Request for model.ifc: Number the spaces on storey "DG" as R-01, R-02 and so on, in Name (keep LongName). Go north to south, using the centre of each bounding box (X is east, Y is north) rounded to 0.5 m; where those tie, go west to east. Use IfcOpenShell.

First a look at what the model holds.

```python
import ifcopenshell
import ifcopenshell.util.element
import ifcopenshell.util.placement

model = ifcopenshell.open("model.ifc")
print(model.schema)
storey = next(s for s in model.by_type("IfcBuildingStorey") if s.Name == "DG")
spaces = [e for e in ifcopenshell.util.element.get_decomposition(storey) if e.is_a("IfcSpace")]
for e in sorted(spaces, key=lambda e: e.id()):
    origin = ifcopenshell.util.placement.get_local_placement(e.ObjectPlacement)[:3, 3]
    print(e.id(), e.Name, e.LongName, origin.round(2) + 0.0, sep=" | ")
```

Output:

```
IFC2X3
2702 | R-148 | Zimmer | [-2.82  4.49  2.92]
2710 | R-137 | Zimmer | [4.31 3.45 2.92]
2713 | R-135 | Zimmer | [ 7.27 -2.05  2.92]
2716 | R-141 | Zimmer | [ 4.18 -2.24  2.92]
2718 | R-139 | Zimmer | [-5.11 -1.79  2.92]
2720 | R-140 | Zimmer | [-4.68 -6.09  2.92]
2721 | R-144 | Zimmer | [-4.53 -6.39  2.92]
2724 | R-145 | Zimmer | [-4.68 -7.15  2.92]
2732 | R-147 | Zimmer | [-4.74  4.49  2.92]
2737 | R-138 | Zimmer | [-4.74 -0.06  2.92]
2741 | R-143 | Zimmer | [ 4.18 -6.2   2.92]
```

```python
import ifcopenshell
import ifcopenshell.geom
import ifcopenshell.util.element
import ifcopenshell.util.shape

model = ifcopenshell.open("model.ifc")
settings = ifcopenshell.geom.settings()
settings.set("use-world-coords", True)


def centre(element):
    shape = ifcopenshell.geom.create_shape(settings, element)
    return ifcopenshell.util.shape.get_bbox_centroid(shape.geometry)


storey = next(s for s in model.by_type("IfcBuildingStorey") if s.Name == "DG")
spaces = [e for e in ifcopenshell.util.element.get_decomposition(storey) if e.is_a("IfcSpace")]

# Insertion points can sit at a corner or the storey origin, so sort by the geometry (in metres).
centres = {e: centre(e) for e in spaces}
spaces.sort(key=lambda e: (-round(centres[e][1] / 0.5), centres[e][0]))

for i, e in enumerate(spaces, start=1):
    number = f"R-{i:02d}"
    e.Name = number
    print(e.id(), number)

model.write("model-out.ifc")
```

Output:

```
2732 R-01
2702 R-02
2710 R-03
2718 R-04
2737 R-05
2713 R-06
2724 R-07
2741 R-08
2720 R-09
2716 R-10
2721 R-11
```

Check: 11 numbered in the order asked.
